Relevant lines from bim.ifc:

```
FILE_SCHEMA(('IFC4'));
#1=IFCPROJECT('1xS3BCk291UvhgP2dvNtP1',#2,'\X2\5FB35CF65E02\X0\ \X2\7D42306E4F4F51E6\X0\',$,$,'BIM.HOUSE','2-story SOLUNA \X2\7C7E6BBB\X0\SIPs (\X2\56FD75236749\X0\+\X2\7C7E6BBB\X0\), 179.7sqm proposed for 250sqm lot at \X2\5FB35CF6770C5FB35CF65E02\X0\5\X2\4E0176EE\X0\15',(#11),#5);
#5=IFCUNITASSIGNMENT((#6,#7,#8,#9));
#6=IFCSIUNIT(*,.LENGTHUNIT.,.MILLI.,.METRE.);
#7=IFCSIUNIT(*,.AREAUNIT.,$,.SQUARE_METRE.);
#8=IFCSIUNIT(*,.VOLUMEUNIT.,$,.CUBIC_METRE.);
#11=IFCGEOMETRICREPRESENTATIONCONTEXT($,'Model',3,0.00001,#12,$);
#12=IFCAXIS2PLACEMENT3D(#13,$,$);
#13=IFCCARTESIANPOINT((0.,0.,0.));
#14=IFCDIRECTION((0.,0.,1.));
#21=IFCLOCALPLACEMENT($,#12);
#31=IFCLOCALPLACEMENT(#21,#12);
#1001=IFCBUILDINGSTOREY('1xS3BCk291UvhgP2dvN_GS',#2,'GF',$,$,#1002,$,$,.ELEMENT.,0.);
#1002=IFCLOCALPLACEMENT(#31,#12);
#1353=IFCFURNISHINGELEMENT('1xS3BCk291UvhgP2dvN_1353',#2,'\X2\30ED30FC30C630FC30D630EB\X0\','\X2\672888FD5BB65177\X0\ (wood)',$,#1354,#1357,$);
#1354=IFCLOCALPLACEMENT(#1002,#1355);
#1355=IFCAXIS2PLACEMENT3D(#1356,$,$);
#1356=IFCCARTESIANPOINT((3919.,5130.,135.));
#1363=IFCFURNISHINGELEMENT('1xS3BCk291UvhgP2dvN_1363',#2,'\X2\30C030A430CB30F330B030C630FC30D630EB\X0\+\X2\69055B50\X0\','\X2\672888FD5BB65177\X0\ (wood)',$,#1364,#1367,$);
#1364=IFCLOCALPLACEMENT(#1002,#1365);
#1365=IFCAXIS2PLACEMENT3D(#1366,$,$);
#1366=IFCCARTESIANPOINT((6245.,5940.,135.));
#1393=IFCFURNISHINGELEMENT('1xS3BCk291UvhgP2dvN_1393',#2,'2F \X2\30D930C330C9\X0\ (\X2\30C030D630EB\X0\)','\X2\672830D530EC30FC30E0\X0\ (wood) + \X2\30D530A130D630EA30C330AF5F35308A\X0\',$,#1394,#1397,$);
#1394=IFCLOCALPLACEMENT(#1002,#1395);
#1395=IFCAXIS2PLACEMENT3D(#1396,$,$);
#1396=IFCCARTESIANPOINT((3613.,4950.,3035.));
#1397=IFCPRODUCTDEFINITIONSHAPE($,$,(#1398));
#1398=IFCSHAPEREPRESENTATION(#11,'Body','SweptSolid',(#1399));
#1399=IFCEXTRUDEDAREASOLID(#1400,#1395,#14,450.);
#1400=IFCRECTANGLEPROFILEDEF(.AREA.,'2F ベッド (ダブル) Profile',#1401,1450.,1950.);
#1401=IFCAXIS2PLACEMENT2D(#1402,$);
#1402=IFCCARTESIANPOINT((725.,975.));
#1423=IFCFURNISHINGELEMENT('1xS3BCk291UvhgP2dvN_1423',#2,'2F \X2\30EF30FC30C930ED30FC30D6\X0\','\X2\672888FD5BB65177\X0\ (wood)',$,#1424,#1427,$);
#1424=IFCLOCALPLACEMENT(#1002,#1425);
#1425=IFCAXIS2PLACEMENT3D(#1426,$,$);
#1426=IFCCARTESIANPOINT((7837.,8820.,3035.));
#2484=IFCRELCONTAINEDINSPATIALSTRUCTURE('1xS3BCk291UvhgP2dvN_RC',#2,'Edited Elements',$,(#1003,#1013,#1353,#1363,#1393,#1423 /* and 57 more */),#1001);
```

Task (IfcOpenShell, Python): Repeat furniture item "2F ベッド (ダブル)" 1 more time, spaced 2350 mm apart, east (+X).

```python
import numpy as np
import ifcopenshell
import ifcopenshell.api.geometry
import ifcopenshell.api.root
import ifcopenshell.util.element
import ifcopenshell.util.placement
import ifcopenshell.util.unit

model = ifcopenshell.open("bim.ifc")
unit_scale = ifcopenshell.util.unit.calculate_unit_scale(model)


def reuse_history(source, copy):
    """copy_class also copies each property set's owner history, people and application; keep the originals."""
    for rel in copy.IsDefinedBy:
        if rel.is_a("IfcRelDefinesByProperties") and (history := rel.RelatingPropertyDefinition.OwnerHistory):
            rel.RelatingPropertyDefinition.OwnerHistory = source.OwnerHistory
            ifcopenshell.util.element.remove_deep2(model, history)


source = model.by_id(1393)
base = ifcopenshell.util.placement.get_local_placement(source.ObjectPlacement)
step = np.array([1.0, 0.0, 0.0]) * 2.35 / unit_scale

for i in range(1, 2):
    copy = ifcopenshell.api.root.copy_class(model, product=source)
    copy.Representation = ifcopenshell.util.element.copy_deep(
        model, source.Representation, exclude=["IfcGeometricRepresentationContext", "IfcRepresentationMap"]
    )
    reuse_history(source, copy)
    matrix = base.copy()
    matrix[:3, 3] += i * step
    print("added at", matrix[:3, 3].round(3) + 0.0)
    ifcopenshell.api.geometry.edit_object_placement(model, product=copy, matrix=matrix, is_si=False)

model.write("bim-out.ifc")
```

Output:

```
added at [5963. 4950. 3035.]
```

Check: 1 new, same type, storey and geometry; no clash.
